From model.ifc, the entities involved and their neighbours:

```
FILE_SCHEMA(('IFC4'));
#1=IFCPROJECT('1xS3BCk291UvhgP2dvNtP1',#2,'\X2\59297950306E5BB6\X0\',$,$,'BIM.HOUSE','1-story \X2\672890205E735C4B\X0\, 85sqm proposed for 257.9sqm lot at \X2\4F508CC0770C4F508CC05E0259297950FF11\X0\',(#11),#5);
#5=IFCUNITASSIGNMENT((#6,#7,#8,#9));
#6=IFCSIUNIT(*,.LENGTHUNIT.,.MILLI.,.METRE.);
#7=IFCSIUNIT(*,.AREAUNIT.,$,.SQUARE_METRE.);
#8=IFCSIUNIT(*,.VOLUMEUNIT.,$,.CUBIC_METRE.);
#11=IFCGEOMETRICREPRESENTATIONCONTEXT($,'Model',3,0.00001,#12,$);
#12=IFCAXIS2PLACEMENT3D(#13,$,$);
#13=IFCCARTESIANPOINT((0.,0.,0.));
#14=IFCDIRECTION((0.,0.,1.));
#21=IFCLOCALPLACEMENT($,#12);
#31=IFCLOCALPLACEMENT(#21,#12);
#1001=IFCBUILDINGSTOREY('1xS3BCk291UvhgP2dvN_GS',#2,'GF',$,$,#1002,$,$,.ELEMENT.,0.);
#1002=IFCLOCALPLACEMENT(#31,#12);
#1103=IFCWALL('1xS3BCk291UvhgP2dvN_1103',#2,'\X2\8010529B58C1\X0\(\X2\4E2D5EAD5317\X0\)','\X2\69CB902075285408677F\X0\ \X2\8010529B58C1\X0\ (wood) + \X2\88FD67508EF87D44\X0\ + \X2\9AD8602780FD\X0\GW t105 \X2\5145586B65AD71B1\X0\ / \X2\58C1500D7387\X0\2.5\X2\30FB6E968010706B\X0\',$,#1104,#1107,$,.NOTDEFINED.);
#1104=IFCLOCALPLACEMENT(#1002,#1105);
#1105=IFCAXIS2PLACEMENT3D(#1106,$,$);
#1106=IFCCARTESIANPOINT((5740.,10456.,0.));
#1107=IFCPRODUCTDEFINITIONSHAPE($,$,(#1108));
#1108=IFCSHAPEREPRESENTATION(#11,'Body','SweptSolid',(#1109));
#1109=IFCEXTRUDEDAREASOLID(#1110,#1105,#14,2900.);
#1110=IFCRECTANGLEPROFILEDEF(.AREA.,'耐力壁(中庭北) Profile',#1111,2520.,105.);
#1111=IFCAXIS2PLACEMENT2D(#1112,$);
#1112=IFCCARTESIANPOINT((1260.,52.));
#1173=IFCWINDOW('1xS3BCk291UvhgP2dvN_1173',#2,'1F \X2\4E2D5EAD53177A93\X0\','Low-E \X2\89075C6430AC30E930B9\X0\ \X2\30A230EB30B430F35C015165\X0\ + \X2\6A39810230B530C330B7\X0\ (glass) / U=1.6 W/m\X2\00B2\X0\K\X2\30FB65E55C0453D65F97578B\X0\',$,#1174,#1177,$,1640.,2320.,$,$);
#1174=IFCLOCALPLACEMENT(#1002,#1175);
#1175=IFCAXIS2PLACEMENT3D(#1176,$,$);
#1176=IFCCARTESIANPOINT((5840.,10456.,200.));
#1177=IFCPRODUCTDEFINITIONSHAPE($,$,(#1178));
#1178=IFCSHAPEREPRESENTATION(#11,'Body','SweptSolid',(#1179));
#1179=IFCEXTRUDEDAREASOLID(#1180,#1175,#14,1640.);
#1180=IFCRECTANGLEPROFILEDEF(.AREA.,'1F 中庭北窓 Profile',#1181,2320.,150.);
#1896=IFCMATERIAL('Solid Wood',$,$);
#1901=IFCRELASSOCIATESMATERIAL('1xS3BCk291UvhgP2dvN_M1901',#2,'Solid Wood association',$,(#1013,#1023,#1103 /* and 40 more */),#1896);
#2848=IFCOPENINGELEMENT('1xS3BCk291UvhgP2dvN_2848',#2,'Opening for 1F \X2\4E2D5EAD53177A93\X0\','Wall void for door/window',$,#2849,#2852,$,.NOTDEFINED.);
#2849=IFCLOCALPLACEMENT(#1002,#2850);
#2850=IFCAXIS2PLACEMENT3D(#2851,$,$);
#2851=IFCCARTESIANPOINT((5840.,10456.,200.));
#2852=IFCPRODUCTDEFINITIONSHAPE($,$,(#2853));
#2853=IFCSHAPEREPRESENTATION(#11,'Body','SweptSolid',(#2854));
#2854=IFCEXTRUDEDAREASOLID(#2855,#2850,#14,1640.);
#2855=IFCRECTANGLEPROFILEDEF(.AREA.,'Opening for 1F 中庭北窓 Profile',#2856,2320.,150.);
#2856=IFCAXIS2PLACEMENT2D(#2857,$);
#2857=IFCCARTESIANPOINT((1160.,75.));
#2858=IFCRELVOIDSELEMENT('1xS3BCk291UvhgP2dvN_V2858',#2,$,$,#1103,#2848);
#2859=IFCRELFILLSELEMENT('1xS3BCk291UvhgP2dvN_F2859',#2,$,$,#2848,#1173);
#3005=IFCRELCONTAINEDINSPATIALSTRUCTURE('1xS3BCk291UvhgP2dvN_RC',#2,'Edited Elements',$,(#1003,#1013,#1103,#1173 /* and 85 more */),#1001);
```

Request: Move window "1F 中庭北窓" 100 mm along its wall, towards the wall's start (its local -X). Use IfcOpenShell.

```python
import ifcopenshell
import ifcopenshell.api.geometry
import ifcopenshell.util.placement

model = ifcopenshell.open("model.ifc")

window = model.by_guid("1xS3BCk291UvhgP2dvN_1173")
opening = window.FillsVoids[0].RelatingOpeningElement
wall = opening.VoidsElements[0].RelatingBuildingElement

wall_matrix = ifcopenshell.util.placement.get_local_placement(wall.ObjectPlacement)
shift = wall_matrix[:3, 0] * -100.0
before = ifcopenshell.util.placement.get_local_placement(window.ObjectPlacement)[:3, 3].copy()

# The window is not placed relative to its opening, so move both.
for product in (opening, window):
    matrix = ifcopenshell.util.placement.get_local_placement(product.ObjectPlacement)
    matrix[:3, 3] += shift
    ifcopenshell.api.geometry.edit_object_placement(model, product=product, matrix=matrix, is_si=False)

after = ifcopenshell.util.placement.get_local_placement(window.ObjectPlacement)[:3, 3]
print("window moved by", (after - before).round(3) + 0.0)

model.write("model_updated.ifc")
```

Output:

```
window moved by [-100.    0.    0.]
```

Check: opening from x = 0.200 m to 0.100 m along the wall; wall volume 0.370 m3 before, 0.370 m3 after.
